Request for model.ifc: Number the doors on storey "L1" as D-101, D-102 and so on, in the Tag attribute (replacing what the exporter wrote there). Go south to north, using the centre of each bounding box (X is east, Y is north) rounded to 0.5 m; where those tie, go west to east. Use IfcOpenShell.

First a look at what the model holds.

```python
import ifcopenshell
import ifcopenshell.util.element
import ifcopenshell.util.placement

model = ifcopenshell.open("model.ifc")
print(model.schema)
storey = next(s for s in model.by_type("IfcBuildingStorey") if s.Name == "L1")
doors = [e for e in ifcopenshell.util.element.get_decomposition(storey) if e.is_a("IfcDoor")]
for e in sorted(doors, key=lambda e: e.id()):
    origin = ifcopenshell.util.placement.get_local_placement(e.ObjectPlacement)[:3, 3]
    print(e.id(), e.Tag, e.Name, origin.round(2) + 0.0, sep=" | ")
```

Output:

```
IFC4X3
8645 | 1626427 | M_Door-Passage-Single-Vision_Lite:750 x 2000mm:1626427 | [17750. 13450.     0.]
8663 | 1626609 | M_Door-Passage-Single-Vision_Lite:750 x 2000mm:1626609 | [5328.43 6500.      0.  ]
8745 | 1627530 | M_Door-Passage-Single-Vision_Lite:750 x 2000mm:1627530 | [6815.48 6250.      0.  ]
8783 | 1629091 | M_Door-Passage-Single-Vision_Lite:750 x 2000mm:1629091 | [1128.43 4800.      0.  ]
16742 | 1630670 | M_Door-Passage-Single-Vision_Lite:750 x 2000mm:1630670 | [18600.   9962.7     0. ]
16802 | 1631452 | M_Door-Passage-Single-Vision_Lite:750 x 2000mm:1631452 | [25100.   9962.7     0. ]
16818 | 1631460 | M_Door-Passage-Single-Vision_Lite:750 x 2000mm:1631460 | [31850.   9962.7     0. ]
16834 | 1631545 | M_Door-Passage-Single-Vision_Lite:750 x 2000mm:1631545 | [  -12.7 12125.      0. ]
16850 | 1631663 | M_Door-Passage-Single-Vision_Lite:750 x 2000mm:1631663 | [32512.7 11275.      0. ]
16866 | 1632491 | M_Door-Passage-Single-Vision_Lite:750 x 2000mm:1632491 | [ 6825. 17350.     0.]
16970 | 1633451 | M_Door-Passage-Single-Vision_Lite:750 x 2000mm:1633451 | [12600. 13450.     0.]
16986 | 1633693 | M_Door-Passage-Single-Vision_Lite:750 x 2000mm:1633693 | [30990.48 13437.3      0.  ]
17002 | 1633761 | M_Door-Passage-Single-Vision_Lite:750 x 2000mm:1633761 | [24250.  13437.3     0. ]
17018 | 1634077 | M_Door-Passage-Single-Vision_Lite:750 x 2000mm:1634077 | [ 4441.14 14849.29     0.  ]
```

```python
import ifcopenshell
import ifcopenshell.geom
import ifcopenshell.util.element
import ifcopenshell.util.shape

model = ifcopenshell.open("model.ifc")
settings = ifcopenshell.geom.settings()
settings.set("use-world-coords", True)


def centre(element):
    shape = ifcopenshell.geom.create_shape(settings, element)
    return ifcopenshell.util.shape.get_bbox_centroid(shape.geometry)


storey = next(s for s in model.by_type("IfcBuildingStorey") if s.Name == "L1")
doors = [e for e in ifcopenshell.util.element.get_decomposition(storey) if e.is_a("IfcDoor")]

# Insertion points can sit at a corner or the storey origin, so sort by the geometry (in metres).
centres = {e: centre(e) for e in doors}
doors.sort(key=lambda e: (round(centres[e][1] / 0.5), centres[e][0]))

for i, e in enumerate(doors, start=1):
    number = f"D-1{i:02d}"
    e.Tag = number
    print(e.id(), number)

model.write("model_v2.ifc")
```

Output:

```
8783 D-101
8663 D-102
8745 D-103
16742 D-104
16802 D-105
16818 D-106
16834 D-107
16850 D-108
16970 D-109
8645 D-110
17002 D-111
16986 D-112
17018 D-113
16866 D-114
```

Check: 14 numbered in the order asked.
